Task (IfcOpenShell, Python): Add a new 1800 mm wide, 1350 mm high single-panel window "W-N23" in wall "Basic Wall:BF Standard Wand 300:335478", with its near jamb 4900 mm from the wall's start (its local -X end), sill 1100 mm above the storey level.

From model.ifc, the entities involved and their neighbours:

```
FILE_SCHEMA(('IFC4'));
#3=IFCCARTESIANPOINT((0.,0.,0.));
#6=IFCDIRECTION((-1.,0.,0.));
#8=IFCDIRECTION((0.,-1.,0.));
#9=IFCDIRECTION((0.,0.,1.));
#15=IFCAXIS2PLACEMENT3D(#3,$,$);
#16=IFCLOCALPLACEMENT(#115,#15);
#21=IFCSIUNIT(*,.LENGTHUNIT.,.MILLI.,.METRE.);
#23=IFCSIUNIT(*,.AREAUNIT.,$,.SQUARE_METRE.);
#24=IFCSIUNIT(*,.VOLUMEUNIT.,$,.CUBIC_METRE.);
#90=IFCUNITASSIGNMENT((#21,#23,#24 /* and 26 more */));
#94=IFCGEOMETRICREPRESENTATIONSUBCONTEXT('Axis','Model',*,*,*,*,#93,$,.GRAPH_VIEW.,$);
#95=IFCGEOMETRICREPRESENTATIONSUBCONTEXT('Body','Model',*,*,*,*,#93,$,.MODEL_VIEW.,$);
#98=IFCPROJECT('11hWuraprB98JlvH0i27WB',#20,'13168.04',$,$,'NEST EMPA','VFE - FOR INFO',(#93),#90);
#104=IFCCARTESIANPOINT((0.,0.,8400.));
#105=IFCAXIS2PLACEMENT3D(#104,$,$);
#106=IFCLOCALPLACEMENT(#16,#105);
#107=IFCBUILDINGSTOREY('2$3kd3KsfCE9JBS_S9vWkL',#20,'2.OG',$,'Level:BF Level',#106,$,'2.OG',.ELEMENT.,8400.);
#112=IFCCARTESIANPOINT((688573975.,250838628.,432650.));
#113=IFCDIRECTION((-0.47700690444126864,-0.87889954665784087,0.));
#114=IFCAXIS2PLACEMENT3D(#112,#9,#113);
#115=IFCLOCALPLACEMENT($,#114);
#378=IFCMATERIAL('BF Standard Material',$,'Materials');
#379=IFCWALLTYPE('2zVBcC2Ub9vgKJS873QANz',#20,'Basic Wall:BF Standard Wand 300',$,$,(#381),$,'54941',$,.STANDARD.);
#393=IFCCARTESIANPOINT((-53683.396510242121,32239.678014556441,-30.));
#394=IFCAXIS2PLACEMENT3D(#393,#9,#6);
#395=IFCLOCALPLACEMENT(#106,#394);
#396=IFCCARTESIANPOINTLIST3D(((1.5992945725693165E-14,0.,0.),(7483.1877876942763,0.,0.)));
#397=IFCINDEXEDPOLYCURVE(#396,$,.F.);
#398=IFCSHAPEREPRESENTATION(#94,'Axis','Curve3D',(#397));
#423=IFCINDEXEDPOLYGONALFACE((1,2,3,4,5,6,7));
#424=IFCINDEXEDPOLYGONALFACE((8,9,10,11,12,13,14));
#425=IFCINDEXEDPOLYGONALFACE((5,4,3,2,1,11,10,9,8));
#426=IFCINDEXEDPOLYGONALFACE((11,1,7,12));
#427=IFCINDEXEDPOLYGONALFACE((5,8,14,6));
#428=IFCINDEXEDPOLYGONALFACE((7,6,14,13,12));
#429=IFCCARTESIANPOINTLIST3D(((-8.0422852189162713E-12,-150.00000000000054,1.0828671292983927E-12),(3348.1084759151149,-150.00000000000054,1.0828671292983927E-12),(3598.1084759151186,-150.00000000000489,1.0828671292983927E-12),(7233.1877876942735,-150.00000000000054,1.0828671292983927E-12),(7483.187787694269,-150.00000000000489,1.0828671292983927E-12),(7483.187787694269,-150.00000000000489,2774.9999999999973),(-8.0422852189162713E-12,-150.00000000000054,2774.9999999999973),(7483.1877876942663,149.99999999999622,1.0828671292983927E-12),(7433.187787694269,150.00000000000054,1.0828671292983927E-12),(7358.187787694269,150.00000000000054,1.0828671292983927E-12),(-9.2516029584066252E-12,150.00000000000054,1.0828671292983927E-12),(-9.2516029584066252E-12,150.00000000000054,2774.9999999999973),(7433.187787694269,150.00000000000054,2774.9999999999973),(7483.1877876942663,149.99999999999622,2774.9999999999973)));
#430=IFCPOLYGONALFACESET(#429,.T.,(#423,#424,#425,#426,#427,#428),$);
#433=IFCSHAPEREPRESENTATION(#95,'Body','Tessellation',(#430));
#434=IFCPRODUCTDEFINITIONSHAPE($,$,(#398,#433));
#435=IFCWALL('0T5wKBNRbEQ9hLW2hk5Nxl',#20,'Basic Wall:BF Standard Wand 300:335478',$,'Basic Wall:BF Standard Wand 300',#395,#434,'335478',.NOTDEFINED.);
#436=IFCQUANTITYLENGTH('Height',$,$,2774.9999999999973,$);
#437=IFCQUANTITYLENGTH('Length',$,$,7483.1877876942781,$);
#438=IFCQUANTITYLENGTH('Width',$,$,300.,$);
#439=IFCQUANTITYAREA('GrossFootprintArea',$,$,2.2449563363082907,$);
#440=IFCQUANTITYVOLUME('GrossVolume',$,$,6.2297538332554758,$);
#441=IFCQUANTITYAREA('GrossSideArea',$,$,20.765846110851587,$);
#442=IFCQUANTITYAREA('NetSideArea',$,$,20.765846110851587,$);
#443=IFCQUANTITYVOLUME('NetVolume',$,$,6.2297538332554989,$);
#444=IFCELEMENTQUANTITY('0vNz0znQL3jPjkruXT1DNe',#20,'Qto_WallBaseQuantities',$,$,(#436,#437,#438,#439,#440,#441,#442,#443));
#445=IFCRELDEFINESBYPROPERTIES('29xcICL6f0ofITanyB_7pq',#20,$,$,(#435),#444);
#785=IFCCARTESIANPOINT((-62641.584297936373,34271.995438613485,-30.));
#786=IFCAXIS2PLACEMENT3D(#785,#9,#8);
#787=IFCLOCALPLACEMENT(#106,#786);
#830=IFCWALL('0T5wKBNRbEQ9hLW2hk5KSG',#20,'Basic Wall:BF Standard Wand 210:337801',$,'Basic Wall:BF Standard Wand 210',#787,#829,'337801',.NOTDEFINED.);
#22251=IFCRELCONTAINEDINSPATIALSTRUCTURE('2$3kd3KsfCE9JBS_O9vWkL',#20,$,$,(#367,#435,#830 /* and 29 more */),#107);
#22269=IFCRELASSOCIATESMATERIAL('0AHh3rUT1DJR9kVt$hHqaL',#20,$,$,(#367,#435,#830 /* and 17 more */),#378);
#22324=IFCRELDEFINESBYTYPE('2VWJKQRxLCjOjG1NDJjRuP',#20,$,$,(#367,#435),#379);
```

```python
import numpy as np
import ifcopenshell
import ifcopenshell.api.feature
import ifcopenshell.api.geometry
import ifcopenshell.api.pset
import ifcopenshell.api.root
import ifcopenshell.api.spatial
import ifcopenshell.geom
import ifcopenshell.util.element
import ifcopenshell.util.placement
import ifcopenshell.util.representation
import ifcopenshell.util.shape
import ifcopenshell.util.unit

model = ifcopenshell.open("model.ifc")
unit_scale = ifcopenshell.util.unit.calculate_unit_scale(model)
area_scale = ifcopenshell.util.unit.calculate_unit_scale(model, "AREAUNIT")
volume_scale = ifcopenshell.util.unit.calculate_unit_scale(model, "VOLUMEUNIT")
settings = ifcopenshell.geom.settings()


def volume(element):
    """Net volume in cubic metres, openings subtracted."""
    shape = ifcopenshell.geom.create_shape(settings, element)
    return ifcopenshell.util.shape.get_volume(shape.geometry)


wall = model.by_guid("0T5wKBNRbEQ9hLW2hk5Nxl")
storey = ifcopenshell.util.element.get_container(wall, ifc_class="IfcBuildingStorey")
context = ifcopenshell.util.representation.get_context(model, "Model", "Body", "MODEL_VIEW")
before = volume(wall)

width, height, from_end, sill = 1.8, 1.35, 4.9, 1.1  # metres

# The wall runs along its own X axis, and the end named is its -X end.
wall_shape = ifcopenshell.geom.create_shape(settings, wall)
x, y, z = ifcopenshell.util.shape.get_vertices(wall_shape.geometry).T
start = x.min() + from_end
face, thickness = float(y.min()), float(y.max() - y.min())
wall_matrix = ifcopenshell.util.placement.get_local_placement(wall.ObjectPlacement)
level = ifcopenshell.util.placement.get_local_placement(storey.ObjectPlacement)[2, 3]


def in_wall(x, y):
    """Placement at x, y metres in the wall's axes, at sill height."""
    matrix = wall_matrix.copy()
    matrix[:, 3] = wall_matrix @ np.array([x / unit_scale, y / unit_scale, 0.0, 1.0])
    matrix[2, 3] = level + sill / unit_scale
    return matrix


# Opening: a box that overshoots both wall faces by 50 mm.
opening = ifcopenshell.api.root.create_entity(model, ifc_class="IfcOpeningElement", predefined_type="OPENING")
box = ifcopenshell.api.geometry.add_wall_representation(
    model, context=context, length=width, height=height, thickness=thickness + 0.1
)
ifcopenshell.api.geometry.assign_representation(model, product=opening, representation=box)
ifcopenshell.api.geometry.edit_object_placement(model, product=opening, matrix=in_wall(start, face - 0.05), is_si=False)
ifcopenshell.api.feature.add_feature(model, feature=opening, element=wall)

window = ifcopenshell.api.root.create_entity(model, ifc_class="IfcWindow", name="W-N23", predefined_type="WINDOW")
window.OverallWidth, window.OverallHeight = width / unit_scale, height / unit_scale
window.PartitioningType = "SINGLE_PANEL"
body = ifcopenshell.api.geometry.add_window_representation(
    model,
    context=context,
    overall_width=window.OverallWidth,
    overall_height=window.OverallHeight,
    partition_type="SINGLE_PANEL",
)
ifcopenshell.api.geometry.assign_representation(model, product=window, representation=body)
ifcopenshell.api.spatial.assign_container(model, products=[window], relating_structure=storey)
ifcopenshell.api.feature.add_filling(model, opening=opening, element=window)

# Centre the window in the wall's thickness.
ifcopenshell.api.geometry.edit_object_placement(model, product=window, matrix=in_wall(start, face), is_si=False)
window_shape = ifcopenshell.geom.create_shape(settings, window)
depth = ifcopenshell.util.shape.get_vertices(window_shape.geometry)[:, 1]
offset = face + thickness / 2 - (depth.min() + depth.max()) / 2
ifcopenshell.api.geometry.edit_object_placement(model, product=window, matrix=in_wall(start, offset), is_si=False)

after = volume(wall)

# Update the wall's stored quantities.
qto = model.by_id(ifcopenshell.util.element.get_pset(wall, "Qto_WallBaseQuantities", should_inherit=False)["id"])
ifcopenshell.api.pset.edit_qto(model, qto=qto, properties={
    "NetSideArea": after / thickness / area_scale,
    "NetVolume": after / volume_scale,
})

print(f"wall volume {before:.3f} -> {after:.3f} m3")

model.write("model-out.ifc")
```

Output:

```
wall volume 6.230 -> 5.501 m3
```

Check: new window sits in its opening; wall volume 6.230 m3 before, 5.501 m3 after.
